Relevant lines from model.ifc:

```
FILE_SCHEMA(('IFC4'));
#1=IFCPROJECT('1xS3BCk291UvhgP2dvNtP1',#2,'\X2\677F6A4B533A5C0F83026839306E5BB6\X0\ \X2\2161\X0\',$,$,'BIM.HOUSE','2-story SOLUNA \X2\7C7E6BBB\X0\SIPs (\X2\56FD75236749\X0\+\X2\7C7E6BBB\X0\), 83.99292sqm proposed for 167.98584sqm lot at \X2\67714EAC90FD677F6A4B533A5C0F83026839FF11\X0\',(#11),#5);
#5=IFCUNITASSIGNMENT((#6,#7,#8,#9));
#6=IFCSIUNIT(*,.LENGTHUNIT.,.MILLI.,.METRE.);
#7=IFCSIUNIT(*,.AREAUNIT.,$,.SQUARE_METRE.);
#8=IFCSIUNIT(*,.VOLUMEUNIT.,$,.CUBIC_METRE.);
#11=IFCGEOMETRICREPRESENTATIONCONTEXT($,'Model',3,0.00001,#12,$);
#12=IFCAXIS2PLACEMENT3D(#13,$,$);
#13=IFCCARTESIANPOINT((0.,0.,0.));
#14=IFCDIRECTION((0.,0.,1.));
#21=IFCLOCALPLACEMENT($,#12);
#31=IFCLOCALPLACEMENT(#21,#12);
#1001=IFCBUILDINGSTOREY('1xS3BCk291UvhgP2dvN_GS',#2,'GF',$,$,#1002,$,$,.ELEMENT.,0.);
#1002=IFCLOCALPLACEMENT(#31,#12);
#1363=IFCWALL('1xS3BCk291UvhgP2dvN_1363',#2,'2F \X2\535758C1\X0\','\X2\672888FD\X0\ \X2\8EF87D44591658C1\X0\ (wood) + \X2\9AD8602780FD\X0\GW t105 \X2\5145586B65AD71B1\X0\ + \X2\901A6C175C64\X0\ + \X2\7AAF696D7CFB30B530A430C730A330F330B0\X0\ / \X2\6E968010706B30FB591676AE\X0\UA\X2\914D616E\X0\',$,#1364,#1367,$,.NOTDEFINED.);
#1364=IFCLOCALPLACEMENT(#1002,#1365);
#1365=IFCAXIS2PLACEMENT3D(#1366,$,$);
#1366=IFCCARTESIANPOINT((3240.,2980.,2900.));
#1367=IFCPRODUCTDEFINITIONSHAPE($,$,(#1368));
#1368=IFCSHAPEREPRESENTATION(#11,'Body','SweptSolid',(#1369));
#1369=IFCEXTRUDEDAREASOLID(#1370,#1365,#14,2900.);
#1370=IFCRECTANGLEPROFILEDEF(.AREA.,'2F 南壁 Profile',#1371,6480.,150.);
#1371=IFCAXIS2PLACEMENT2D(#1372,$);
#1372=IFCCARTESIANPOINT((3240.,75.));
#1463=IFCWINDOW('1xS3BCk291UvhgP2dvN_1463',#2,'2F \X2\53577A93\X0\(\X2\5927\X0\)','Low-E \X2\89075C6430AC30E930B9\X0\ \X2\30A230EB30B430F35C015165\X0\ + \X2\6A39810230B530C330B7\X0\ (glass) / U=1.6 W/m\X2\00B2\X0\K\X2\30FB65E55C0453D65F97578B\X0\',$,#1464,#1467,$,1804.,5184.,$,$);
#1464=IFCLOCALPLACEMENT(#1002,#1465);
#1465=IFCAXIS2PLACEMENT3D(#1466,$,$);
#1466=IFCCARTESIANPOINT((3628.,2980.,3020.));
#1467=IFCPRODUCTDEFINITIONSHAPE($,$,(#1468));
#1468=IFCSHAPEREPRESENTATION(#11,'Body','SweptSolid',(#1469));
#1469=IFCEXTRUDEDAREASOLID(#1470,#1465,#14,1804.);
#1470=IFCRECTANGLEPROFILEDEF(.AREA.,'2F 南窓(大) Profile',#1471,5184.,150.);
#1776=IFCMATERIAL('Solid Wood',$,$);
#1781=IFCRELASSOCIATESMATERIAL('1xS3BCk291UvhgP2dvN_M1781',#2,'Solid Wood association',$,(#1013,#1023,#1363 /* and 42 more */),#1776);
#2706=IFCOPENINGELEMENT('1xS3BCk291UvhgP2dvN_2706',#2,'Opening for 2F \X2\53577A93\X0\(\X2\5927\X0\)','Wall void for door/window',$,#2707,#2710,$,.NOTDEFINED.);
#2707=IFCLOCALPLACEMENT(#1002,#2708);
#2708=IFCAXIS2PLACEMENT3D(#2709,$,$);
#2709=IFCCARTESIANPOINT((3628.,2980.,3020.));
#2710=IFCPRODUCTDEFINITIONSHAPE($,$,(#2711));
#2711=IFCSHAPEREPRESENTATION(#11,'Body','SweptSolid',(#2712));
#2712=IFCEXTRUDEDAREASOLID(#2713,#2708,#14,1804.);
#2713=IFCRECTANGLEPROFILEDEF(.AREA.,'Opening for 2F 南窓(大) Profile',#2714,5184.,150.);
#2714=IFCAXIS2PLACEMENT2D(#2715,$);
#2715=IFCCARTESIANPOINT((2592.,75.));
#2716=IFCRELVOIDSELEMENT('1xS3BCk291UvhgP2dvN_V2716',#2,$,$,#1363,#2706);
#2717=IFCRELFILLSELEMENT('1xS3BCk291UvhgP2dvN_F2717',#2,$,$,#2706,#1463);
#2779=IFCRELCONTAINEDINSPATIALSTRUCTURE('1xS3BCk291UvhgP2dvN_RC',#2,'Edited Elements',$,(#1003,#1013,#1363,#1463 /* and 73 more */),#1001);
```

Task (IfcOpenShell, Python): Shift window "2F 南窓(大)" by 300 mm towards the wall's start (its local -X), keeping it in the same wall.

```python
import ifcopenshell
import ifcopenshell.api.geometry
import ifcopenshell.util.placement
import ifcopenshell.util.unit

model = ifcopenshell.open("model.ifc")
unit_scale = ifcopenshell.util.unit.calculate_unit_scale(model)

window = model.by_guid("1xS3BCk291UvhgP2dvN_1463")
opening = window.FillsVoids[0].RelatingOpeningElement
wall = opening.VoidsElements[0].RelatingBuildingElement

wall_matrix = ifcopenshell.util.placement.get_local_placement(wall.ObjectPlacement)
shift = wall_matrix[:3, 0] * -0.3 / unit_scale
before = ifcopenshell.util.placement.get_local_placement(window.ObjectPlacement)[:3, 3].copy()

# The window is not placed relative to its opening, so move both.
for product in (opening, window):
    matrix = ifcopenshell.util.placement.get_local_placement(product.ObjectPlacement)
    matrix[:3, 3] += shift
    ifcopenshell.api.geometry.edit_object_placement(model, product=product, matrix=matrix, is_si=False)

after = ifcopenshell.util.placement.get_local_placement(window.ObjectPlacement)[:3, 3]
print("window moved by", (after - before).round(3) + 0.0)

model.write("model_edited.ifc")
```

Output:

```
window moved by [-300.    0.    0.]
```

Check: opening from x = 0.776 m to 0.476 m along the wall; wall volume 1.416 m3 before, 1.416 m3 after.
